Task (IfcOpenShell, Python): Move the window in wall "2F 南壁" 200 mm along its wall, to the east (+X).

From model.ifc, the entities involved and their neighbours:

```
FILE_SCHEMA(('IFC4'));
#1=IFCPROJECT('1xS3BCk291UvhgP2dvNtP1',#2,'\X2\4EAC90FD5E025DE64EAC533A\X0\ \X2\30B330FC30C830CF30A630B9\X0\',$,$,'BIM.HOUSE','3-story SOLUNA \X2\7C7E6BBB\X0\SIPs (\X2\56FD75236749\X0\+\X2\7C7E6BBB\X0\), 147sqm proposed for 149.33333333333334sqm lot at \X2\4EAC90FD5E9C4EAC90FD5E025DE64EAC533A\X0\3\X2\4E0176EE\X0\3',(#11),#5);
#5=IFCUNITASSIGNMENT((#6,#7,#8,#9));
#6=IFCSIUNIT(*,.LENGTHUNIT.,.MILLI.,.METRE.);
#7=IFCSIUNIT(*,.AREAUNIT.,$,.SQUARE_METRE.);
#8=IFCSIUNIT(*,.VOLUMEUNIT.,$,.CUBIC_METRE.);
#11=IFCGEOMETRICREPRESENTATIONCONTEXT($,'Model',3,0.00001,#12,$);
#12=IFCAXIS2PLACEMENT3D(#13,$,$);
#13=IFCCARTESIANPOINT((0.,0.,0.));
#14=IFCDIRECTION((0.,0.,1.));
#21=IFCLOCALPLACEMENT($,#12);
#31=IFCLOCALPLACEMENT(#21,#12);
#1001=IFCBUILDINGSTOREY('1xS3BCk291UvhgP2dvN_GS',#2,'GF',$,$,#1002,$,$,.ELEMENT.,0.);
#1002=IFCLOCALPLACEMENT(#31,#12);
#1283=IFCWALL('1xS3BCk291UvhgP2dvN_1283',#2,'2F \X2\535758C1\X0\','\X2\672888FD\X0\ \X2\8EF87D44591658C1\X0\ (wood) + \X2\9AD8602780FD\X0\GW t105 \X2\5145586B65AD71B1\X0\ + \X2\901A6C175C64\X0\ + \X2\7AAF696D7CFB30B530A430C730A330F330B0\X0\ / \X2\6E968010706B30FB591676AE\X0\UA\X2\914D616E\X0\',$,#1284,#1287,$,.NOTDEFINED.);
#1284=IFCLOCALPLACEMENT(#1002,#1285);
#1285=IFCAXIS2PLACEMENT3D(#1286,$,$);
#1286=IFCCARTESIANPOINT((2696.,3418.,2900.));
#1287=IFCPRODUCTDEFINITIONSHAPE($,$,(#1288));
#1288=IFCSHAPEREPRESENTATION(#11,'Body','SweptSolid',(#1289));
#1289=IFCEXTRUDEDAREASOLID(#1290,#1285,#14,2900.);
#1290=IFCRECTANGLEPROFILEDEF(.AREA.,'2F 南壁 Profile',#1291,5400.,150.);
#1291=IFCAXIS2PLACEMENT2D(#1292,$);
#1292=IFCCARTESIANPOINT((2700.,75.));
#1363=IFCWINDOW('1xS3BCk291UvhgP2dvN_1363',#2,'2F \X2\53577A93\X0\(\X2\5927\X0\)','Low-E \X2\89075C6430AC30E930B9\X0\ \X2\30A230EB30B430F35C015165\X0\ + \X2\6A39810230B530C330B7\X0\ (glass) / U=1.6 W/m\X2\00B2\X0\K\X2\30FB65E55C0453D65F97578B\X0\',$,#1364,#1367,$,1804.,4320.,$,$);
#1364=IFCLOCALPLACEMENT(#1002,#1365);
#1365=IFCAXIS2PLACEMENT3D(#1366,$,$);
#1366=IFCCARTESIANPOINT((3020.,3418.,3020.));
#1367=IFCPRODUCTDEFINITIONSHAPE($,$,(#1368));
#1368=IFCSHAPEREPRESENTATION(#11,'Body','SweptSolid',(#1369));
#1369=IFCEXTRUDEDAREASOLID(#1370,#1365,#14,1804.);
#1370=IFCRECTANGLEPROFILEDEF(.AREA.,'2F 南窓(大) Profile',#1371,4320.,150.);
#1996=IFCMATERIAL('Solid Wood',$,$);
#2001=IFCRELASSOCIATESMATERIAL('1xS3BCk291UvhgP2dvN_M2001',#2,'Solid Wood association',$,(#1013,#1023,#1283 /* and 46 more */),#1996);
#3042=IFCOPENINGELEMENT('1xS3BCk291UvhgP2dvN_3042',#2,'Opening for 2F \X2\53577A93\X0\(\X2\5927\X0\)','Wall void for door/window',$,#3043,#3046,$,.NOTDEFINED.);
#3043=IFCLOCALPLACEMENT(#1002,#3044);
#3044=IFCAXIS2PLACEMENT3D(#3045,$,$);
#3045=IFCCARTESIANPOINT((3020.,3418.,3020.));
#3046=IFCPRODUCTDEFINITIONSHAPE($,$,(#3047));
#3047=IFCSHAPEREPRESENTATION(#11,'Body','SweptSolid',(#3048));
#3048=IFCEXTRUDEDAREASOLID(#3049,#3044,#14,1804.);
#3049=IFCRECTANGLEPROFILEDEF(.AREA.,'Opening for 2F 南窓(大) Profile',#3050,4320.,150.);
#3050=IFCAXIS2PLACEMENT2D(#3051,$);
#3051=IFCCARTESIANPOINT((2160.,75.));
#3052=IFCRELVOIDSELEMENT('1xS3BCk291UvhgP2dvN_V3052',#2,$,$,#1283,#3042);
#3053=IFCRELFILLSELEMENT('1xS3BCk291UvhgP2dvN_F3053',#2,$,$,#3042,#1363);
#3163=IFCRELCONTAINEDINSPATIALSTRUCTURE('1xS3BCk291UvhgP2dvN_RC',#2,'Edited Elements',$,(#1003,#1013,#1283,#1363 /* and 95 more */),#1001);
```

```python
import ifcopenshell
import ifcopenshell.api.geometry
import ifcopenshell.util.placement
import ifcopenshell.util.unit

model = ifcopenshell.open("model.ifc")
unit_scale = ifcopenshell.util.unit.calculate_unit_scale(model)

window = model.by_guid("1xS3BCk291UvhgP2dvN_1363")
opening = window.FillsVoids[0].RelatingOpeningElement
wall = opening.VoidsElements[0].RelatingBuildingElement

wall_matrix = ifcopenshell.util.placement.get_local_placement(wall.ObjectPlacement)
shift = wall_matrix[:3, 0] * 0.2 / unit_scale
before = ifcopenshell.util.placement.get_local_placement(window.ObjectPlacement)[:3, 3].copy()

# The window is not placed relative to its opening, so move both.
for product in (opening, window):
    matrix = ifcopenshell.util.placement.get_local_placement(product.ObjectPlacement)
    matrix[:3, 3] += shift
    ifcopenshell.api.geometry.edit_object_placement(model, product=product, matrix=matrix, is_si=False)

after = ifcopenshell.util.placement.get_local_placement(window.ObjectPlacement)[:3, 3]
print("window moved by", (after - before).round(3) + 0.0)

model.write("model-out.ifc")
```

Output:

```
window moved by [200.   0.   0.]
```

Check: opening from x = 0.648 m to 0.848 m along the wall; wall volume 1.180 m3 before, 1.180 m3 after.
